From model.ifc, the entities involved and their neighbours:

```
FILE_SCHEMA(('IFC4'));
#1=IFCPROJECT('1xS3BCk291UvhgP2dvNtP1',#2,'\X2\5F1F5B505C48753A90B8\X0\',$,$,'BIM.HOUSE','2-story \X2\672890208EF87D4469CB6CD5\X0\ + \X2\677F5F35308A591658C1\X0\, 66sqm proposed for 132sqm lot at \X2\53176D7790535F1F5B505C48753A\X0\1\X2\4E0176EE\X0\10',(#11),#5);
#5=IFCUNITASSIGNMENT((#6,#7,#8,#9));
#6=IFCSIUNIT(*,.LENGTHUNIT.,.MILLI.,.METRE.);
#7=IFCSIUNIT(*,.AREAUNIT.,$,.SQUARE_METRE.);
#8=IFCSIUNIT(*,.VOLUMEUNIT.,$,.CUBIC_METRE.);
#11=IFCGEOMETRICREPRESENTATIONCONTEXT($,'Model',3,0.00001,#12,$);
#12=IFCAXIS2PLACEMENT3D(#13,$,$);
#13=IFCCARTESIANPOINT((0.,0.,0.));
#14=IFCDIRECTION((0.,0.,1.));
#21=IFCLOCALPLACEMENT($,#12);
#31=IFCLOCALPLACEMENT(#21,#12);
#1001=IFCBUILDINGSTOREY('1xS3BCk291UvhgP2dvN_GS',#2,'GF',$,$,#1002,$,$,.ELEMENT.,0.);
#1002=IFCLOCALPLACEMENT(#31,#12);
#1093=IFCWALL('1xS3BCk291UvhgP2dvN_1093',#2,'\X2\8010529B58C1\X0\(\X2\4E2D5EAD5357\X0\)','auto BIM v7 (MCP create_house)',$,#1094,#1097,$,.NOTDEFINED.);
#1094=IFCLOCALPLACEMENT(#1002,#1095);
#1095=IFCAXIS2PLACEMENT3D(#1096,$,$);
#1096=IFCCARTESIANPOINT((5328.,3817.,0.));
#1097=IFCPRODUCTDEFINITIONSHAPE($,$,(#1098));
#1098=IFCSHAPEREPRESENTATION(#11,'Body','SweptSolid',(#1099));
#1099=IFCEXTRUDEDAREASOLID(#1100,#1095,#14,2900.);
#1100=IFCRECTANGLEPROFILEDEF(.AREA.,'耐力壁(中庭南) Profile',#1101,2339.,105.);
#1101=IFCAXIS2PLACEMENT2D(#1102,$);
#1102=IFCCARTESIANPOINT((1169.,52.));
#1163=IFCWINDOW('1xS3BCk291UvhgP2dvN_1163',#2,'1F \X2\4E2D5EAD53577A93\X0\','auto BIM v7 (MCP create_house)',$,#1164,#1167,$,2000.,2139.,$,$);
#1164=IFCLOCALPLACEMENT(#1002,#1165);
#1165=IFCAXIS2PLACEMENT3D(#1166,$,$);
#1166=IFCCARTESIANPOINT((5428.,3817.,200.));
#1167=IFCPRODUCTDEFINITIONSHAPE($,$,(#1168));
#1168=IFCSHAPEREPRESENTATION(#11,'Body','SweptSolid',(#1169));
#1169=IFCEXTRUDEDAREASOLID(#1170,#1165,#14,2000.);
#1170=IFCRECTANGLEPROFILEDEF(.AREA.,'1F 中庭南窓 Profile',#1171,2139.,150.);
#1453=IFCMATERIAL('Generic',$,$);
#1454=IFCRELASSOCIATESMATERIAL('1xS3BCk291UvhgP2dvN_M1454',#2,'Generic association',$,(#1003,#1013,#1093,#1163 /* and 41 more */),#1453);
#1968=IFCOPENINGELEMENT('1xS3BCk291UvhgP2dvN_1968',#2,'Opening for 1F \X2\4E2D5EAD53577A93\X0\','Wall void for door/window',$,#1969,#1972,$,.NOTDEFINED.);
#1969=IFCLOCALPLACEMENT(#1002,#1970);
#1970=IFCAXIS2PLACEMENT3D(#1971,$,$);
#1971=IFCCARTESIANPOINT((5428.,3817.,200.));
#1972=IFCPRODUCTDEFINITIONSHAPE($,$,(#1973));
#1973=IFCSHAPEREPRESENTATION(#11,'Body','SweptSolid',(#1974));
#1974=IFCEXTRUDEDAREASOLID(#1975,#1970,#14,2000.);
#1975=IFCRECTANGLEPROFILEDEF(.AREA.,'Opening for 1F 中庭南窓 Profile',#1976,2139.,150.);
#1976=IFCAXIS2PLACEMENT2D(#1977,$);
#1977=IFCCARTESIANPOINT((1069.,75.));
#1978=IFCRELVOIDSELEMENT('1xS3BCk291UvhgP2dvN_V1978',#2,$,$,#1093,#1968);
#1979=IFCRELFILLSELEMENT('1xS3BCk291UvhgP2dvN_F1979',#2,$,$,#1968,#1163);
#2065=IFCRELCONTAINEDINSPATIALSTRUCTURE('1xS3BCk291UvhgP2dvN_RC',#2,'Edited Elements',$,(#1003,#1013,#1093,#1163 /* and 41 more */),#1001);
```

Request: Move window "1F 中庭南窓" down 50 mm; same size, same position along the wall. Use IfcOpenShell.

```python
import numpy as np
import ifcopenshell
import ifcopenshell.api.geometry
import ifcopenshell.util.placement
import ifcopenshell.util.unit

model = ifcopenshell.open("model.ifc")
unit_scale = ifcopenshell.util.unit.calculate_unit_scale(model)

window = model.by_guid("1xS3BCk291UvhgP2dvN_1163")
opening = window.FillsVoids[0].RelatingOpeningElement
dz = -50.0

shift = np.array([0.0, 0.0, dz])
# The window is not placed relative to its opening, so move both.
for product in (opening, window):
    matrix = ifcopenshell.util.placement.get_local_placement(product.ObjectPlacement)
    matrix[:3, 3] += shift
    ifcopenshell.api.geometry.edit_object_placement(model, product=product, matrix=matrix, is_si=False)

print(f"moved by {dz * unit_scale:+.3f} m")

model.write("model_edited.ifc")
```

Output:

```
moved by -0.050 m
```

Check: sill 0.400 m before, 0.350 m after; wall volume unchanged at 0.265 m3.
